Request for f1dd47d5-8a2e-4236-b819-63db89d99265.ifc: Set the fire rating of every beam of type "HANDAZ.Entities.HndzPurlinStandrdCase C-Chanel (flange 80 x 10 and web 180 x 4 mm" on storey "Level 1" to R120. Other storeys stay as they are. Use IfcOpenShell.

First a look at what the model holds.

```python
import ifcopenshell
import ifcopenshell.util.element

model = ifcopenshell.open("f1dd47d5-8a2e-4236-b819-63db89d99265.ifc")
print(model.schema)
storey = next(s for s in model.by_type("IfcBuildingStorey") if s.Name == "Level 1")
beams = [e for e in ifcopenshell.util.element.get_decomposition(storey) if e.is_a("IfcBeam")]
seen = {}
for e in beams:
    element_type = ifcopenshell.util.element.get_type(e)
    key = (element_type.Name if element_type != e and element_type else None, ifcopenshell.util.element.get_pset(e, "Pset_BeamCommon", "FireRating"))
    seen[key] = seen.get(key, 0) + 1
for (name, value), count in sorted(seen.items(), key=str):
    print(count, "x", name, "|", value)
```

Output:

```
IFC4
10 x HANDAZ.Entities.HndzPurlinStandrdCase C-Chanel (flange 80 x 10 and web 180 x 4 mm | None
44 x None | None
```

```python
import ifcopenshell
import ifcopenshell.api.pset
import ifcopenshell.util.element

model = ifcopenshell.open("f1dd47d5-8a2e-4236-b819-63db89d99265.ifc")

storey = next(s for s in model.by_type("IfcBuildingStorey") if s.Name == "Level 1")
beams = [e for e in ifcopenshell.util.element.get_decomposition(storey) if e.is_a("IfcBeam")]

count = 0
for e in beams:
    element_type = ifcopenshell.util.element.get_type(e)
    if element_type in (None, e) or element_type.Name != "HANDAZ.Entities.HndzPurlinStandrdCase C-Chanel (flange 80 x 10 and web 180 x 4 mm":
        continue
    # add_pset returns the element's existing set when there is one.
    pset = ifcopenshell.api.pset.add_pset(model, product=e, name="Pset_BeamCommon")
    ifcopenshell.api.pset.edit_pset(model, pset=pset, properties={"FireRating": "R120"})
    count += 1

print(count, "beams updated")

model.write("f1dd47d5-8a2e-4236-b819-63db89d99265_edited.ifc")
```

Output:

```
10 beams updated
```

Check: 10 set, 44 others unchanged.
